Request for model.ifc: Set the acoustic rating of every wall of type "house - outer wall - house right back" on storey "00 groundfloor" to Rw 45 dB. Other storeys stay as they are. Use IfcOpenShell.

First a look at what the model holds.

```python
import ifcopenshell
import ifcopenshell.util.element

model = ifcopenshell.open("model.ifc")
print(model.schema)
storey = next(s for s in model.by_type("IfcBuildingStorey") if s.Name == "00 groundfloor")
walls = [e for e in ifcopenshell.util.element.get_decomposition(storey) if e.is_a("IfcWall")]
seen = {}
for e in walls:
    element_type = ifcopenshell.util.element.get_type(e)
    key = (element_type.Name if element_type != e and element_type else None, ifcopenshell.util.element.get_pset(e, "Pset_WallCommon", "AcousticRating"))
    seen[key] = seen.get(key, 0) + 1
for (name, value), count in sorted(seen.items(), key=str):
    print(count, "x", name, "|", value)
```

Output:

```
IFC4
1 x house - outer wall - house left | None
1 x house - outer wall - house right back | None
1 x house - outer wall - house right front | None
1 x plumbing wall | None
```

```python
import ifcopenshell
import ifcopenshell.api.pset
import ifcopenshell.util.element

model = ifcopenshell.open("model.ifc")

storey = next(s for s in model.by_type("IfcBuildingStorey") if s.Name == "00 groundfloor")
walls = [e for e in ifcopenshell.util.element.get_decomposition(storey) if e.is_a("IfcWall")]

count = 0
for e in walls:
    element_type = ifcopenshell.util.element.get_type(e)
    if element_type in (None, e) or element_type.Name != "house - outer wall - house right back":
        continue
    # add_pset returns the element's existing set when there is one.
    pset = ifcopenshell.api.pset.add_pset(model, product=e, name="Pset_WallCommon")
    ifcopenshell.api.pset.edit_pset(model, pset=pset, properties={"AcousticRating": "Rw 45 dB"})
    count += 1

print(count, "walls updated")

model.write("model_v2.ifc")
```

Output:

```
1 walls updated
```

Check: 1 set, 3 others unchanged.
